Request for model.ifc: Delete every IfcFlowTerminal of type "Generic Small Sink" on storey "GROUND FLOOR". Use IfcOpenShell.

First a look at what the model holds.

```python
import ifcopenshell
import ifcopenshell.util.element

model = ifcopenshell.open("model.ifc")
print(model.schema)
storey = next(s for s in model.by_type("IfcBuildingStorey") if s.Name == "GROUND FLOOR")
terminals = [e for e in ifcopenshell.util.element.get_decomposition(storey) if e.is_a("IfcFlowTerminal")]
seen = {}
for e in terminals:
    element_type = ifcopenshell.util.element.get_type(e)
    name = element_type.Name if element_type not in (None, e) else None
    seen[name] = seen.get(name, 0) + 1
for name, count in sorted(seen.items(), key=str):
    print(count, "x", name)
```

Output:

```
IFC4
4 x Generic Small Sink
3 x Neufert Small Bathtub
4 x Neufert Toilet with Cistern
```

```python
import ifcopenshell
import ifcopenshell.api.root
import ifcopenshell.util.element

model = ifcopenshell.open("model.ifc")

storey = next(s for s in model.by_type("IfcBuildingStorey") if s.Name == "GROUND FLOOR")
terminals = [e for e in ifcopenshell.util.element.get_decomposition(storey) if e.is_a("IfcFlowTerminal")]
targets = [e for e in terminals if (t := ifcopenshell.util.element.get_type(e)) not in (None, e) and t.Name == "Generic Small Sink"]

for e in targets:
    ifcopenshell.api.root.remove_product(model, product=e)
print(len(targets), "removed")

model.write("model_v2.ifc")
```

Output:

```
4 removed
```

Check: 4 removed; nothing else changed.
